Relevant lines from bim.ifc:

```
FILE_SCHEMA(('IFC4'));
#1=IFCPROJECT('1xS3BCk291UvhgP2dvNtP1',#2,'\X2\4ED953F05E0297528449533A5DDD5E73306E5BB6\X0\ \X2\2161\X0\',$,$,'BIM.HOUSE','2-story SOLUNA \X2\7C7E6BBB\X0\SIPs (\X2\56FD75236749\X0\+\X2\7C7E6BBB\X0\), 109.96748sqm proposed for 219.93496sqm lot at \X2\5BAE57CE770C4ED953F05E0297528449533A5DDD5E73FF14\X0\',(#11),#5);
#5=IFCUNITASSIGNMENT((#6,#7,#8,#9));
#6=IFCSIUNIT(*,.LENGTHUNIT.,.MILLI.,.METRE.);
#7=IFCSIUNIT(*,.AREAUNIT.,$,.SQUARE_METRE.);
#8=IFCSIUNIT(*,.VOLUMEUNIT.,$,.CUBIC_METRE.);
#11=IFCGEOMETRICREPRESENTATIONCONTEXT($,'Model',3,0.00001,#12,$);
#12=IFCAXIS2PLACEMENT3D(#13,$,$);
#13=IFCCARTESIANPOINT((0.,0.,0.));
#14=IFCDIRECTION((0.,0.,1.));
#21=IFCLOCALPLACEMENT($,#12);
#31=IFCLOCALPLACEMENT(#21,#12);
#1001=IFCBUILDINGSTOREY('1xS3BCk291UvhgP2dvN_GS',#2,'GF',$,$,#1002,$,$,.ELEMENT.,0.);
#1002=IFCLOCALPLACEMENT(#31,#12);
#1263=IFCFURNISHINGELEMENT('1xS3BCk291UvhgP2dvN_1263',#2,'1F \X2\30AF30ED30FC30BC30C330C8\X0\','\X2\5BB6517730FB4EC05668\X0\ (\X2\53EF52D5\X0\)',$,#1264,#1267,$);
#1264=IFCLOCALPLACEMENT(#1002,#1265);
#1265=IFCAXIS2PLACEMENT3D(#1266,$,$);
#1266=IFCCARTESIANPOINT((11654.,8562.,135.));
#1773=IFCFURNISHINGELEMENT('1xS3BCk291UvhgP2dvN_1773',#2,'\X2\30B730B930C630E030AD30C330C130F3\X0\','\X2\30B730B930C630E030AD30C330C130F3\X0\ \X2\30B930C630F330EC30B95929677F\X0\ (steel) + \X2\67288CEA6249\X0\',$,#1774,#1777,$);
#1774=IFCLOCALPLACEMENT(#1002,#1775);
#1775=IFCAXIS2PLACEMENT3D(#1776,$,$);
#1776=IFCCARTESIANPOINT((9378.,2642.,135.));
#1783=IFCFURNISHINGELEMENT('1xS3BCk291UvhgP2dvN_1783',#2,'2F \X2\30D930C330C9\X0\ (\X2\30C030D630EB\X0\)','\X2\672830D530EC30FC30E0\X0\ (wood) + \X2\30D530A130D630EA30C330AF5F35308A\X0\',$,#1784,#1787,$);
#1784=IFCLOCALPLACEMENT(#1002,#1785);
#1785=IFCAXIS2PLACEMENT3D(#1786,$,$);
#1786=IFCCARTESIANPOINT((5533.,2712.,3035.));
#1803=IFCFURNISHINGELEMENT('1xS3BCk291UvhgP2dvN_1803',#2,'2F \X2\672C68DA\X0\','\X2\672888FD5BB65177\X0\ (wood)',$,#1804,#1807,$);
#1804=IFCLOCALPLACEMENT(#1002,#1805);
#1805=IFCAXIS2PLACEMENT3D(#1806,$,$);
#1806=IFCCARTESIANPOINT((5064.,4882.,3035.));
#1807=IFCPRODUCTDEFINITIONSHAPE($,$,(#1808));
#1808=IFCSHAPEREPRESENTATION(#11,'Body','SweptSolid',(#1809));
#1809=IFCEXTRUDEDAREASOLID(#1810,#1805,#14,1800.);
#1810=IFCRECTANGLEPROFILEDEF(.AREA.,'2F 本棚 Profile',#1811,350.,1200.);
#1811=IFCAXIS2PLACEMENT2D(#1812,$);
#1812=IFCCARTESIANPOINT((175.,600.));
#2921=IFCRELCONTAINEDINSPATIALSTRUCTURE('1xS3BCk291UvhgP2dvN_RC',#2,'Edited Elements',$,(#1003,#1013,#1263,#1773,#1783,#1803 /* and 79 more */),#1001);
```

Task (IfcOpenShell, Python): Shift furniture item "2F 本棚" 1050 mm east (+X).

```python
import ifcopenshell
import ifcopenshell.api.geometry
import ifcopenshell.util.placement
import ifcopenshell.util.unit

model = ifcopenshell.open("bim.ifc")
unit_scale = ifcopenshell.util.unit.calculate_unit_scale(model)

item = model.by_guid("1xS3BCk291UvhgP2dvN_1803")
matrix = ifcopenshell.util.placement.get_local_placement(item.ObjectPlacement)
matrix[0, 3] += 1.05 / unit_scale
ifcopenshell.api.geometry.edit_object_placement(model, product=item, matrix=matrix, is_si=False)

print(ifcopenshell.util.placement.get_local_placement(item.ObjectPlacement).round(3) + 0.0)

model.write("bim-out.ifc")
```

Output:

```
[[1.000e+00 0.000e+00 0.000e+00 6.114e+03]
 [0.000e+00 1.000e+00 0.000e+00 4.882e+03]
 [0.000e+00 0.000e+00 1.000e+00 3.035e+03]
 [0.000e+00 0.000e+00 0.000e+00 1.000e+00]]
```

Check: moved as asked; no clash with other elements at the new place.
